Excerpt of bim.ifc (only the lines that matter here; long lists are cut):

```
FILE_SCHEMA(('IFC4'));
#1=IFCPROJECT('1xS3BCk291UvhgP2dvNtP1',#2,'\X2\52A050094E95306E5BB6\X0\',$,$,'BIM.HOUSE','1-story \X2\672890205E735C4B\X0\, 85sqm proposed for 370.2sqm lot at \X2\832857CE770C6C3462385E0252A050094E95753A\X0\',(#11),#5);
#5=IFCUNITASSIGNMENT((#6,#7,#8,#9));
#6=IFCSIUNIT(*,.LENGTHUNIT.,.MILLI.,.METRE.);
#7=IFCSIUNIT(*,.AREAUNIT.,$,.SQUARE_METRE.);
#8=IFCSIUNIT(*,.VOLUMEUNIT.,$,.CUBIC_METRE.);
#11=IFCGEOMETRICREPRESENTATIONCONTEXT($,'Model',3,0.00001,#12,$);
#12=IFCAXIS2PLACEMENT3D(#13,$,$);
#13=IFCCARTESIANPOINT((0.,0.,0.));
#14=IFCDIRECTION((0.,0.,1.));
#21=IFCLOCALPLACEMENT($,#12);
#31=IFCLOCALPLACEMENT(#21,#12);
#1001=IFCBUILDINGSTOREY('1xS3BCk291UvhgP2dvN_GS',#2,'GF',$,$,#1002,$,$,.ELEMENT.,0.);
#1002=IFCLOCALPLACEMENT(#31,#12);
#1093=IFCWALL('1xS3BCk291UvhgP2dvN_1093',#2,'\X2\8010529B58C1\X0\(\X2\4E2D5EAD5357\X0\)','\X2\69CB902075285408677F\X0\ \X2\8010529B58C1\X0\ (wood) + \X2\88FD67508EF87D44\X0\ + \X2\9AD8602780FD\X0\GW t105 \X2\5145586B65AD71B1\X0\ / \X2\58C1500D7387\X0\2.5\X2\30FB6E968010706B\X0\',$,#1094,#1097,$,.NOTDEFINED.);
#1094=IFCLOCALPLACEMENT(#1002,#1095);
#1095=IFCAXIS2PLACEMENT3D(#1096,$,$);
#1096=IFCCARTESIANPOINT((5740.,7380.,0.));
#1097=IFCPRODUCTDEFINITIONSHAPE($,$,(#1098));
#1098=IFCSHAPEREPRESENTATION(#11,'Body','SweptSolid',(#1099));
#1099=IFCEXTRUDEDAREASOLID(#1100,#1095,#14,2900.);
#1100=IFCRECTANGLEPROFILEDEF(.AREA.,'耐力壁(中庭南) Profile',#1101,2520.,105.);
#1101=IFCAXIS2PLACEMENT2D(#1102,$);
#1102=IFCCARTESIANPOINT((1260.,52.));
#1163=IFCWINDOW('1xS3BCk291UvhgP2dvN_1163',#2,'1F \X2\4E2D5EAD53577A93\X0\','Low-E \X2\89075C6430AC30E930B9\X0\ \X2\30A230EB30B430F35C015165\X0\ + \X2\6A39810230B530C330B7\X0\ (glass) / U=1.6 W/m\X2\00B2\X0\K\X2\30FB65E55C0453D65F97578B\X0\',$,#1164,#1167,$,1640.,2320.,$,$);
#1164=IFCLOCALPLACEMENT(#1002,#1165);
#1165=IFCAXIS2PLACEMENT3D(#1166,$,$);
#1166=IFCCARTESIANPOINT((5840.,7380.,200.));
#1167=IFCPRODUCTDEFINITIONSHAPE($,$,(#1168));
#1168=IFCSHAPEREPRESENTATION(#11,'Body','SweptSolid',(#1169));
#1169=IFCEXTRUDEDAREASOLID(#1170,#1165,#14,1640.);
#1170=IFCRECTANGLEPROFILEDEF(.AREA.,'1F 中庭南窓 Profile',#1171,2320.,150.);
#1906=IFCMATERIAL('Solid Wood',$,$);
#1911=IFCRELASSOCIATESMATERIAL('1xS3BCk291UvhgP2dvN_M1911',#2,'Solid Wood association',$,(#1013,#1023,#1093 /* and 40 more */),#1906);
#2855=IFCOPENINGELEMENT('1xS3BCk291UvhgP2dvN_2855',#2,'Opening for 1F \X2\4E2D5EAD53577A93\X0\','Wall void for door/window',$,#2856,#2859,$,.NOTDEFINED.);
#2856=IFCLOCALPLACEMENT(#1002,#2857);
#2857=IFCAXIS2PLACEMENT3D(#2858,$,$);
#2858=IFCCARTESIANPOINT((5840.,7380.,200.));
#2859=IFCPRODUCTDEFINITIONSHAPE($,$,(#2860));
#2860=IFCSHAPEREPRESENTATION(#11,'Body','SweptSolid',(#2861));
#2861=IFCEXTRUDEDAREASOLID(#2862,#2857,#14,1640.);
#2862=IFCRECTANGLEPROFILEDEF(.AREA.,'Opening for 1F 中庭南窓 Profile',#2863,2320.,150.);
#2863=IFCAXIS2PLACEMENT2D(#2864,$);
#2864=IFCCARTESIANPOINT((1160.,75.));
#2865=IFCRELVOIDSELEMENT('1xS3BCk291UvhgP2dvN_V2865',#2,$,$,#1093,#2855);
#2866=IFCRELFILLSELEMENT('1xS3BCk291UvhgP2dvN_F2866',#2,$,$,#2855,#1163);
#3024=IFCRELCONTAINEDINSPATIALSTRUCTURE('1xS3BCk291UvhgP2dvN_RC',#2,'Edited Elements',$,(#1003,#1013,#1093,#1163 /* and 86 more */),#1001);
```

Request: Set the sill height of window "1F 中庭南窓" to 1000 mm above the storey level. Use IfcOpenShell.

```python
import numpy as np
import ifcopenshell
import ifcopenshell.api.geometry
import ifcopenshell.geom
import ifcopenshell.util.element
import ifcopenshell.util.placement
import ifcopenshell.util.shape
import ifcopenshell.util.unit

model = ifcopenshell.open("bim.ifc")
unit_scale = ifcopenshell.util.unit.calculate_unit_scale(model)

window = model.by_guid("1xS3BCk291UvhgP2dvN_1163")
opening = window.FillsVoids[0].RelatingOpeningElement
storey = ifcopenshell.util.element.get_container(window, ifc_class="IfcBuildingStorey")
level = ifcopenshell.util.placement.get_local_placement(storey.ObjectPlacement)[2, 3]

# The opening's origin need not be at the sill, so measure its lowest point.
shape = ifcopenshell.geom.create_shape(ifcopenshell.geom.settings(), opening)
bottom = ifcopenshell.util.shape.get_shape_bottom_elevation(shape, shape.geometry) / unit_scale
dz = level + 1 / unit_scale - bottom

shift = np.array([0.0, 0.0, dz])
# The window is not placed relative to its opening, so move both.
for product in (opening, window):
    matrix = ifcopenshell.util.placement.get_local_placement(product.ObjectPlacement)
    matrix[:3, 3] += shift
    ifcopenshell.api.geometry.edit_object_placement(model, product=product, matrix=matrix, is_si=False)

print(f"moved by {dz * unit_scale:+.3f} m")

model.write("bim_edited.ifc")
```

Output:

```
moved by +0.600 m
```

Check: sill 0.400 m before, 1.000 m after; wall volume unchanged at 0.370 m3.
